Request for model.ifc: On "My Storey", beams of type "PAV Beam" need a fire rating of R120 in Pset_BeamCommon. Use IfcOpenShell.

First a look at what the model holds.

```python
import ifcopenshell
import ifcopenshell.util.element

model = ifcopenshell.open("model.ifc")
print(model.schema)
storey = next(s for s in model.by_type("IfcBuildingStorey") if s.Name == "My Storey")
beams = [e for e in ifcopenshell.util.element.get_decomposition(storey) if e.is_a("IfcBeam")]
seen = {}
for e in beams:
    element_type = ifcopenshell.util.element.get_type(e)
    key = (element_type.Name if element_type != e and element_type else None, ifcopenshell.util.element.get_pset(e, "Pset_BeamCommon", "FireRating"))
    seen[key] = seen.get(key, 0) + 1
for (name, value), count in sorted(seen.items(), key=str):
    print(count, "x", name, "|", value)
```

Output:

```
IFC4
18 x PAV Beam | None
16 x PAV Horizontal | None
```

```python
import ifcopenshell
import ifcopenshell.api.pset
import ifcopenshell.util.element

model = ifcopenshell.open("model.ifc")

storey = next(s for s in model.by_type("IfcBuildingStorey") if s.Name == "My Storey")
beams = [e for e in ifcopenshell.util.element.get_decomposition(storey) if e.is_a("IfcBeam")]

count = 0
for e in beams:
    element_type = ifcopenshell.util.element.get_type(e)
    if element_type in (None, e) or element_type.Name != "PAV Beam":
        continue
    # add_pset returns the element's existing set when there is one.
    pset = ifcopenshell.api.pset.add_pset(model, product=e, name="Pset_BeamCommon")
    ifcopenshell.api.pset.edit_pset(model, pset=pset, properties={"FireRating": "R120"})
    count += 1

print(count, "beams updated")

model.write("model_v2.ifc")
```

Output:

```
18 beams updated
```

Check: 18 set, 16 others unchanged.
